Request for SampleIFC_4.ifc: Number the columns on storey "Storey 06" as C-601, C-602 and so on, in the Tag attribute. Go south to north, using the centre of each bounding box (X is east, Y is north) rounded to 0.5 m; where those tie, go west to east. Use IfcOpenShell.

First a look at what the model holds.

```python
import ifcopenshell
import ifcopenshell.util.element
import ifcopenshell.util.placement

model = ifcopenshell.open("SampleIFC_4.ifc")
print(model.schema)
storey = next(s for s in model.by_type("IfcBuildingStorey") if s.Name == "Storey 06")
columns = [e for e in ifcopenshell.util.element.get_decomposition(storey) if e.is_a("IfcColumn")]
for e in sorted(columns, key=lambda e: e.id()):
    origin = ifcopenshell.util.placement.get_local_placement(e.ObjectPlacement)[:3, 3]
    print(e.id(), e.Tag, e.Name, origin.round(2) + 0.0, sep=" | ")
```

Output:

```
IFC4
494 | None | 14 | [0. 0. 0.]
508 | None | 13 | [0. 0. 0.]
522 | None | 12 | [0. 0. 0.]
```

```python
import ifcopenshell
import ifcopenshell.geom
import ifcopenshell.util.element
import ifcopenshell.util.shape

model = ifcopenshell.open("SampleIFC_4.ifc")
settings = ifcopenshell.geom.settings()
settings.set("use-world-coords", True)


def centre(element):
    shape = ifcopenshell.geom.create_shape(settings, element)
    return ifcopenshell.util.shape.get_bbox_centroid(shape.geometry)


storey = next(s for s in model.by_type("IfcBuildingStorey") if s.Name == "Storey 06")
columns = [e for e in ifcopenshell.util.element.get_decomposition(storey) if e.is_a("IfcColumn")]

# Insertion points can sit at a corner or the storey origin, so sort by the geometry (in metres).
centres = {e: centre(e) for e in columns}
columns.sort(key=lambda e: (round(centres[e][1] / 0.5), centres[e][0]))

for i, e in enumerate(columns, start=1):
    number = f"C-6{i:02d}"
    e.Tag = number
    print(e.id(), number)

model.write("SampleIFC_4_edited.ifc")
```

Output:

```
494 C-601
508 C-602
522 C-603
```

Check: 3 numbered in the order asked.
